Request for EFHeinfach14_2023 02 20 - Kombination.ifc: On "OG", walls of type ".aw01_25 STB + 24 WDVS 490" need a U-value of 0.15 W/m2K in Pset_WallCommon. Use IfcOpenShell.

First a look at what the model holds.

```python
import ifcopenshell
import ifcopenshell.util.element

model = ifcopenshell.open("EFHeinfach14_2023 02 20 - Kombination.ifc")
print(model.schema)
storey = next(s for s in model.by_type("IfcBuildingStorey") if s.Name == "OG")
walls = [e for e in ifcopenshell.util.element.get_decomposition(storey) if e.is_a("IfcWall")]
seen = {}
for e in walls:
    element_type = ifcopenshell.util.element.get_type(e)
    key = (element_type.Name if element_type != e and element_type else None, ifcopenshell.util.element.get_pset(e, "Pset_WallCommon", "ThermalTransmittance"))
    seen[key] = seen.get(key, 0) + 1
for (name, value), count in sorted(seen.items(), key=str):
    print(count, "x", name, "|", value)
```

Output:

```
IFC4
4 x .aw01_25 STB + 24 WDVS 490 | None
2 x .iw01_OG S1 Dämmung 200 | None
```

```python
import ifcopenshell
import ifcopenshell.api.pset
import ifcopenshell.util.element

model = ifcopenshell.open("EFHeinfach14_2023 02 20 - Kombination.ifc")

storey = next(s for s in model.by_type("IfcBuildingStorey") if s.Name == "OG")
walls = [e for e in ifcopenshell.util.element.get_decomposition(storey) if e.is_a("IfcWall")]

count = 0
for e in walls:
    element_type = ifcopenshell.util.element.get_type(e)
    if element_type in (None, e) or element_type.Name != ".aw01_25 STB + 24 WDVS 490":
        continue
    # add_pset returns the element's existing set when there is one.
    pset = ifcopenshell.api.pset.add_pset(model, product=e, name="Pset_WallCommon")
    ifcopenshell.api.pset.edit_pset(model, pset=pset, properties={"ThermalTransmittance": 0.15})
    count += 1

print(count, "walls updated")

model.write("EFHeinfach14_2023 02 20 - Kombination-out.ifc")
```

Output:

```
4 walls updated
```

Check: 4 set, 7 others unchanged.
